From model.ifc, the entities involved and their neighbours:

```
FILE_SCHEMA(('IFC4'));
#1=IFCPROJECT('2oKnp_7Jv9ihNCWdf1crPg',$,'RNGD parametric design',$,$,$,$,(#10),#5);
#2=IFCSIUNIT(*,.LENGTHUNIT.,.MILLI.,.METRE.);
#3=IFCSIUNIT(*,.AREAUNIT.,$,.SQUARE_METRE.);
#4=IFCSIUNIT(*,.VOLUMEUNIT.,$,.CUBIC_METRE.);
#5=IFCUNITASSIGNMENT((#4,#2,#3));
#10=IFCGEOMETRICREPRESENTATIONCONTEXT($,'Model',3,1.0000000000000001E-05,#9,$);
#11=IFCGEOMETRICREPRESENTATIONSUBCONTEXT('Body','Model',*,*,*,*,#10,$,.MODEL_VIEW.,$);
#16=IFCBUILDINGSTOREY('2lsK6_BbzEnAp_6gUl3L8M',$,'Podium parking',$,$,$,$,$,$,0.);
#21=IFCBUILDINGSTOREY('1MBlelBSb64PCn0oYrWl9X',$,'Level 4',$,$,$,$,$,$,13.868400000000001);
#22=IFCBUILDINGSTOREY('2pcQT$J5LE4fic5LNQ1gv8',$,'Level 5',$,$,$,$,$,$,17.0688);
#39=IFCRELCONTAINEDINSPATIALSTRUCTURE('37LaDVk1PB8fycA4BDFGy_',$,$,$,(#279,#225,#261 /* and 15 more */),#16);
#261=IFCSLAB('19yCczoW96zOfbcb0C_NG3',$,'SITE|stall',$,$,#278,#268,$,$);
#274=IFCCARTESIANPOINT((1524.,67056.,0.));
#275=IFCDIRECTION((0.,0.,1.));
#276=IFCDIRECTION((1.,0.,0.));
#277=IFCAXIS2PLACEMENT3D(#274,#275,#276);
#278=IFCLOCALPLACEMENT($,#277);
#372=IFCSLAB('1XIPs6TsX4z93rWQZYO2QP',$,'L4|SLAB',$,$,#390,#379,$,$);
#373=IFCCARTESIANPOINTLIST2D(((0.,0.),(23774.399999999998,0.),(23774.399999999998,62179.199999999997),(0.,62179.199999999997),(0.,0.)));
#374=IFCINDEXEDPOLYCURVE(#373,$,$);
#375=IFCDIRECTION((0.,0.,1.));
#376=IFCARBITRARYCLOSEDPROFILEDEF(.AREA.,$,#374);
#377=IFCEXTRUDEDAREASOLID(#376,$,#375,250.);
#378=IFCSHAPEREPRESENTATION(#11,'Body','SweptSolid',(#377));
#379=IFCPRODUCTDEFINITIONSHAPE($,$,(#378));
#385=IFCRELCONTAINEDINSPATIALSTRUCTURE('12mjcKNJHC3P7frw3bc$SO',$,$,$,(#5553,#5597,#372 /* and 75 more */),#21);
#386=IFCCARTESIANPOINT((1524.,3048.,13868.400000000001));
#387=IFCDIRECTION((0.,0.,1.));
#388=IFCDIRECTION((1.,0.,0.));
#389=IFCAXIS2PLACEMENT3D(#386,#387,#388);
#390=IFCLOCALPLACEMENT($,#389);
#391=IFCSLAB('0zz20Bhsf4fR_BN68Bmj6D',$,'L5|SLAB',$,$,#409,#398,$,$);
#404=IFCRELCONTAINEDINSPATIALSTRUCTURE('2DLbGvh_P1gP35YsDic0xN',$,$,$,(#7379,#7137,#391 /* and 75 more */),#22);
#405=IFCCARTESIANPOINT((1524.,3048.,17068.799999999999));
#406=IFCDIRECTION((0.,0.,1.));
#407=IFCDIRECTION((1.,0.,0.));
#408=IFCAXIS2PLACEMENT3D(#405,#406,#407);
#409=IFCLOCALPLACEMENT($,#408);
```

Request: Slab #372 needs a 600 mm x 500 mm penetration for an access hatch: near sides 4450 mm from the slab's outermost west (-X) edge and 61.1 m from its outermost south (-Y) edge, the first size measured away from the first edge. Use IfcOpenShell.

```python
import numpy as np
import ifcopenshell
import ifcopenshell.api.feature
import ifcopenshell.api.geometry
import ifcopenshell.api.root
import ifcopenshell.geom
import ifcopenshell.util.placement
import ifcopenshell.util.representation
import ifcopenshell.util.shape
import ifcopenshell.util.unit

model = ifcopenshell.open("model.ifc")
unit_scale = ifcopenshell.util.unit.calculate_unit_scale(model)
settings = ifcopenshell.geom.settings()


def volume(element):
    """Net volume in cubic metres, openings subtracted."""
    shape = ifcopenshell.geom.create_shape(settings, element)
    return ifcopenshell.util.shape.get_volume(shape.geometry)


slab = model.by_guid("1XIPs6TsX4z93rWQZYO2QP")
before = volume(slab)

# Extent in the slab's own axes, in metres. The edges named are its -X and -Y sides.
slab_shape = ifcopenshell.geom.create_shape(settings, slab)
vertices = ifcopenshell.util.shape.get_vertices(slab_shape.geometry)
x_min, y_min, bottom = vertices.min(axis=0)
top = vertices[:, 2].max()

opening = ifcopenshell.api.root.create_entity(model, ifc_class="IfcOpeningElement", name="Access hatch opening", predefined_type="OPENING")
context = ifcopenshell.util.representation.get_context(model, "Model", "Body", "MODEL_VIEW")
width, depth = 0.6, 0.5
outline = [(0.0, 0.0), (width, 0.0), (width, depth), (0.0, depth), (0.0, 0.0)]
# Overshoot both faces by 50 mm so the cut is clean.
shape = ifcopenshell.api.geometry.add_slab_representation(
    model, context=context, depth=top - bottom + 0.1, polyline=outline
)
ifcopenshell.api.geometry.assign_representation(model, product=opening, representation=shape)

matrix = ifcopenshell.util.placement.get_local_placement(slab.ObjectPlacement)
matrix[:, 3] = matrix @ np.append(np.array([x_min + 4.45, y_min + 61.1, bottom - 0.05]) / unit_scale, 1.0)
ifcopenshell.api.geometry.edit_object_placement(model, product=opening, matrix=matrix, is_si=False)
ifcopenshell.api.feature.add_feature(model, feature=opening, element=slab)

after = volume(slab)

print(f"slab volume {before:.3f} -> {after:.3f} m3")

model.write("model_edited.ifc")
```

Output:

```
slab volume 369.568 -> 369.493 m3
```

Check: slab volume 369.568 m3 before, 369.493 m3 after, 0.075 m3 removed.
